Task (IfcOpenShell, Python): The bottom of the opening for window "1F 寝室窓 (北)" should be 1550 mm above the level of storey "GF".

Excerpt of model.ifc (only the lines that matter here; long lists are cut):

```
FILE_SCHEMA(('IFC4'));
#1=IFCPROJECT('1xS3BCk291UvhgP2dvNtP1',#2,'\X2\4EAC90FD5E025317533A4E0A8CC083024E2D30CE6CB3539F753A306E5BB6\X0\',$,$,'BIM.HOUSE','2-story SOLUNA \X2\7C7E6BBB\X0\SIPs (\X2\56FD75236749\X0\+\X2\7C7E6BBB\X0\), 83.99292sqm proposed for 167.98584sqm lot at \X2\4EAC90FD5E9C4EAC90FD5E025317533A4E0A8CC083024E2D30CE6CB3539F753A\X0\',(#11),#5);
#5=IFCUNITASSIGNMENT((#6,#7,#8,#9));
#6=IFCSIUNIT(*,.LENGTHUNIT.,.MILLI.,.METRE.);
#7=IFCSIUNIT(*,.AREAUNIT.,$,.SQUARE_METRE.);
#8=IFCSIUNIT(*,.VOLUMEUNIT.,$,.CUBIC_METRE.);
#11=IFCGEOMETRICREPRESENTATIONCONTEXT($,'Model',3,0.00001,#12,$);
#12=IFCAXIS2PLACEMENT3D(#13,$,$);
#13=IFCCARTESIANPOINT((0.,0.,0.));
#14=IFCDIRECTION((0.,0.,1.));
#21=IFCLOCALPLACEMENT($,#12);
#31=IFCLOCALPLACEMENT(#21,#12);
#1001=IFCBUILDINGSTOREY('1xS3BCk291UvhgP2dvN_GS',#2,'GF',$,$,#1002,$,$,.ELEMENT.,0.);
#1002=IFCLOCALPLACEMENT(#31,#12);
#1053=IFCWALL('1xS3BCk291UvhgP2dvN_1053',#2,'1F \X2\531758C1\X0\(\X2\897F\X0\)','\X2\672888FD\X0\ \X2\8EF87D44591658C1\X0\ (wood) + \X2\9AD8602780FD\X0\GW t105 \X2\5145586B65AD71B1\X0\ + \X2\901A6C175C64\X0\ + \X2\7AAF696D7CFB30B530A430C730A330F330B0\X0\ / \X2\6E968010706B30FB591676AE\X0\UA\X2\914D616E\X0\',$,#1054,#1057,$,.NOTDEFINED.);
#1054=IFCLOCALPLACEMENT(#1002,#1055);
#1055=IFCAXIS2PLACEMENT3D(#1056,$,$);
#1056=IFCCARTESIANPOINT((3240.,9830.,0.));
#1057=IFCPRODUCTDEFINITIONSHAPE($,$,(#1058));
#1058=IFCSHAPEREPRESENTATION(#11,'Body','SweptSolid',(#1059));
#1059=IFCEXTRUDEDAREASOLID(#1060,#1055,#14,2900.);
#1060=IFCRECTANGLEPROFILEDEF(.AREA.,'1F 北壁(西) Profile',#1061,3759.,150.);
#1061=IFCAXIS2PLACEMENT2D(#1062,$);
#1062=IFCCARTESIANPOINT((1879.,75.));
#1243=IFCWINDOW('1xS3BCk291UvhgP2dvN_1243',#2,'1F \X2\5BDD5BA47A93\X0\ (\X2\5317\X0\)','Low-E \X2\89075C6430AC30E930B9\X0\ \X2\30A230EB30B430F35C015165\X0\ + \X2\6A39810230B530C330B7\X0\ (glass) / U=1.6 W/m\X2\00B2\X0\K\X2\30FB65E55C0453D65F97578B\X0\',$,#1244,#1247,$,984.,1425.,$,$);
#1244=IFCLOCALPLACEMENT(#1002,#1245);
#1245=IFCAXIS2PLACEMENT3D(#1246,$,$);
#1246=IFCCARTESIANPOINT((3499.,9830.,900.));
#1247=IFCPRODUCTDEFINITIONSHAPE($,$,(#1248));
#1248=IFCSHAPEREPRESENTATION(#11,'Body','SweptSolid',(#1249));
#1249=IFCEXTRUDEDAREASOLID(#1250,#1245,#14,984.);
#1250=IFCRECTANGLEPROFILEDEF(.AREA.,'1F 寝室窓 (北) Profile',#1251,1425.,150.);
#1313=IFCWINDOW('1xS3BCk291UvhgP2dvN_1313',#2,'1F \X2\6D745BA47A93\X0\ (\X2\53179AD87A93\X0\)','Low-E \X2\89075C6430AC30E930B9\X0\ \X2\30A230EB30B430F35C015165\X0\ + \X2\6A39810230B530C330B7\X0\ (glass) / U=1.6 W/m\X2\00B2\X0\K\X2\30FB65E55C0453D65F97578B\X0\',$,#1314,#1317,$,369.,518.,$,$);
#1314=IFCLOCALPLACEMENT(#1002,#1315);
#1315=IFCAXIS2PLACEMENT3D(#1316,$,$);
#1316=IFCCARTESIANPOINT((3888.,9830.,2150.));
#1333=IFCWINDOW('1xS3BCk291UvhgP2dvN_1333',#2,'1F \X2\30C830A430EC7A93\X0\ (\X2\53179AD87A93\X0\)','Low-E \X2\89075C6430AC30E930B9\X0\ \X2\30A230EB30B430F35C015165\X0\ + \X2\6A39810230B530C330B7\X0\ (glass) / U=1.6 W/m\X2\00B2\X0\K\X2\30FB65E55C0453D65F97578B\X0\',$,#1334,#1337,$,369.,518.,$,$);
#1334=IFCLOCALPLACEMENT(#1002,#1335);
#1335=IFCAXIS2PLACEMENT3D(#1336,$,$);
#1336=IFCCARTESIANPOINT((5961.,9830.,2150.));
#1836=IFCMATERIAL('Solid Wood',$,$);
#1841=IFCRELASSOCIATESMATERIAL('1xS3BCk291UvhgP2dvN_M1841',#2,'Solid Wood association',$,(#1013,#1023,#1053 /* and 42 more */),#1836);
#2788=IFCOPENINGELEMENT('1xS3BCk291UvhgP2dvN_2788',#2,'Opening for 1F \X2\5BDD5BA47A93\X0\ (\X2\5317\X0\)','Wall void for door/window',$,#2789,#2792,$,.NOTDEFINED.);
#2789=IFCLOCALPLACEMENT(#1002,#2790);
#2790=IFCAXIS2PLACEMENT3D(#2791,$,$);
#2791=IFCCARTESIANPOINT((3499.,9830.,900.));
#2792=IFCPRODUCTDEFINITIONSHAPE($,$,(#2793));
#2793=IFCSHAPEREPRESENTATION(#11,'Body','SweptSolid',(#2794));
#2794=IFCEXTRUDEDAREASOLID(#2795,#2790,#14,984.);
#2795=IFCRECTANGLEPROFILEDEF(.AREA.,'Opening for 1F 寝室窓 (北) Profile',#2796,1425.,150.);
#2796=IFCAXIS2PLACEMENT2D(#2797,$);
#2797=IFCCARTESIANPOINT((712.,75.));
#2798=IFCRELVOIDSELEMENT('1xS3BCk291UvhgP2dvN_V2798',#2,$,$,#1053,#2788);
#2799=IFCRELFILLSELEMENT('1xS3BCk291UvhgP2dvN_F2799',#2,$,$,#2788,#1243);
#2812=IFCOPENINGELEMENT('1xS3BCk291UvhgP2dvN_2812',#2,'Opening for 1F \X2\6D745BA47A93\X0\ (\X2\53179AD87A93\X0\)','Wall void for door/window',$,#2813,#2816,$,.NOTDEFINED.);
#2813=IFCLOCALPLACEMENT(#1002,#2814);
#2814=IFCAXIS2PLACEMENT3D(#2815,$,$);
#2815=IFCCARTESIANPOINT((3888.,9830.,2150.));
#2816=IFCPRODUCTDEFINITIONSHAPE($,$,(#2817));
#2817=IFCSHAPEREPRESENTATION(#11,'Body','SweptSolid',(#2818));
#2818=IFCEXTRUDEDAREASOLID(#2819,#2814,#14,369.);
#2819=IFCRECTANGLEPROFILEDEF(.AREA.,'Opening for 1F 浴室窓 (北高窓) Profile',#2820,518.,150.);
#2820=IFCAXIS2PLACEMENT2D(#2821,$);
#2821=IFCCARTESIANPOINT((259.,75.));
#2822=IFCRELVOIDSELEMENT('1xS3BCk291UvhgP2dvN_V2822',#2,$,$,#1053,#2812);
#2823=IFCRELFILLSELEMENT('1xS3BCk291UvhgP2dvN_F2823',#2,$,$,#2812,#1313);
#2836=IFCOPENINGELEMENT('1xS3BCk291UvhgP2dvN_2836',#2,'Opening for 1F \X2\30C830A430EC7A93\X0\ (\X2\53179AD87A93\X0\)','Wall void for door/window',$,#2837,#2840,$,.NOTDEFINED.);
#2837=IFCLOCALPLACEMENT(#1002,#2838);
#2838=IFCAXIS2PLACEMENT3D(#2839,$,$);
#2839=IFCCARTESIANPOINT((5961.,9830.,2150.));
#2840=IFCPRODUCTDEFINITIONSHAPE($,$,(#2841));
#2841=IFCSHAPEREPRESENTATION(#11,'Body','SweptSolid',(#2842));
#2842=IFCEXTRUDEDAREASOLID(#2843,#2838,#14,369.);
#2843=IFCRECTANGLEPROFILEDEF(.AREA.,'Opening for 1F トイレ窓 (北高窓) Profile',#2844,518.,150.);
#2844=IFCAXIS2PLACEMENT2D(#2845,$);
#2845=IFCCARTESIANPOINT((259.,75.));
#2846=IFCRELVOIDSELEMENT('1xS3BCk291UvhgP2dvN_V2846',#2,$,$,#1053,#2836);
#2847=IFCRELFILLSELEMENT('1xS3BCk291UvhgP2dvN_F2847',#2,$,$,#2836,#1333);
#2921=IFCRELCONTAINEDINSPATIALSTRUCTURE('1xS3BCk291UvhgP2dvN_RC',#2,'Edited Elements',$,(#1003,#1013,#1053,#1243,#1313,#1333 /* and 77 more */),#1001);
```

```python
import numpy as np
import ifcopenshell
import ifcopenshell.api.geometry
import ifcopenshell.geom
import ifcopenshell.util.element
import ifcopenshell.util.placement
import ifcopenshell.util.shape
import ifcopenshell.util.unit

model = ifcopenshell.open("model.ifc")
unit_scale = ifcopenshell.util.unit.calculate_unit_scale(model)

window = model.by_guid("1xS3BCk291UvhgP2dvN_1243")
opening = window.FillsVoids[0].RelatingOpeningElement
storey = ifcopenshell.util.element.get_container(window, ifc_class="IfcBuildingStorey")
level = ifcopenshell.util.placement.get_local_placement(storey.ObjectPlacement)[2, 3]

# The opening's origin need not be at the sill, so measure its lowest point.
shape = ifcopenshell.geom.create_shape(ifcopenshell.geom.settings(), opening)
bottom = ifcopenshell.util.shape.get_shape_bottom_elevation(shape, shape.geometry) / unit_scale
dz = level + 1.55 / unit_scale - bottom

shift = np.array([0.0, 0.0, dz])
# The window is not placed relative to its opening, so move both.
for product in (opening, window):
    matrix = ifcopenshell.util.placement.get_local_placement(product.ObjectPlacement)
    matrix[:3, 3] += shift
    ifcopenshell.api.geometry.edit_object_placement(model, product=product, matrix=matrix, is_si=False)

print(f"moved by {dz * unit_scale:+.3f} m")

model.write("model-out.ifc")
```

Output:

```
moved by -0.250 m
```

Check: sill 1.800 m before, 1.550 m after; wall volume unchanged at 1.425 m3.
